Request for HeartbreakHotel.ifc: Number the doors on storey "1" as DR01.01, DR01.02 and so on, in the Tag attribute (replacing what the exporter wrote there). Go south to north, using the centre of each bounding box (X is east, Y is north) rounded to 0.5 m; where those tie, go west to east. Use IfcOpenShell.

First a look at what the model holds.

```python
import ifcopenshell
import ifcopenshell.util.element
import ifcopenshell.util.placement

model = ifcopenshell.open("HeartbreakHotel.ifc")
print(model.schema)
storey = next(s for s in model.by_type("IfcBuildingStorey") if s.Name == "1")
doors = [e for e in ifcopenshell.util.element.get_decomposition(storey) if e.is_a("IfcDoor")]
for e in sorted(doors, key=lambda e: e.id()):
    origin = ifcopenshell.util.placement.get_local_placement(e.ObjectPlacement)[:3, 3]
    print(e.id(), e.Tag, e.Name, origin.round(2) + 0.0, sep=" | ")
```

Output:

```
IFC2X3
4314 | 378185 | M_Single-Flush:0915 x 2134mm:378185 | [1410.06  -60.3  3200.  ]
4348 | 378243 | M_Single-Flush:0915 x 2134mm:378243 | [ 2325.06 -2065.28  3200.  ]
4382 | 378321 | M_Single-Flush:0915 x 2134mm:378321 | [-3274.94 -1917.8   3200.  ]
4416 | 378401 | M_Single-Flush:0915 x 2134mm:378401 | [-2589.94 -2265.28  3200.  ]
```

```python
import ifcopenshell
import ifcopenshell.geom
import ifcopenshell.util.element
import ifcopenshell.util.shape

model = ifcopenshell.open("HeartbreakHotel.ifc")
settings = ifcopenshell.geom.settings()
settings.set("use-world-coords", True)


def centre(element):
    shape = ifcopenshell.geom.create_shape(settings, element)
    return ifcopenshell.util.shape.get_bbox_centroid(shape.geometry)


storey = next(s for s in model.by_type("IfcBuildingStorey") if s.Name == "1")
doors = [e for e in ifcopenshell.util.element.get_decomposition(storey) if e.is_a("IfcDoor")]

# Insertion points can sit at a corner or the storey origin, so sort by the geometry (in metres).
centres = {e: centre(e) for e in doors}
doors.sort(key=lambda e: (round(centres[e][1] / 0.5), centres[e][0]))

for i, e in enumerate(doors, start=1):
    number = f"DR01.{i:02d}"
    e.Tag = number
    print(e.id(), number)

model.write("HeartbreakHotel_rev.ifc")
```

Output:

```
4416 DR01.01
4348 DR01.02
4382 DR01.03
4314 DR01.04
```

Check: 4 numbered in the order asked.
